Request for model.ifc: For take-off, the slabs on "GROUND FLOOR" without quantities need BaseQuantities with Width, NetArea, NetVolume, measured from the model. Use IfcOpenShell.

First a look at what the model holds.

```python
import ifcopenshell
import ifcopenshell.util.element
import ifcopenshell.util.unit

model = ifcopenshell.open("model.ifc")
print(model.schema)
for unit_type in ("LENGTHUNIT", "AREAUNIT", "VOLUMEUNIT"):
    print(unit_type, ifcopenshell.util.unit.calculate_unit_scale(model, unit_type))
storey = next(s for s in model.by_type("IfcBuildingStorey") if s.Name == "GROUND FLOOR")
slabs = [e for e in ifcopenshell.util.element.get_decomposition(storey) if e.is_a("IfcSlab")]
for e in sorted(slabs, key=lambda e: e.id()):
    print(e.id(), e.is_a(), e.Name, list(ifcopenshell.util.element.get_psets(e, qtos_only=True)), sep=" | ")
```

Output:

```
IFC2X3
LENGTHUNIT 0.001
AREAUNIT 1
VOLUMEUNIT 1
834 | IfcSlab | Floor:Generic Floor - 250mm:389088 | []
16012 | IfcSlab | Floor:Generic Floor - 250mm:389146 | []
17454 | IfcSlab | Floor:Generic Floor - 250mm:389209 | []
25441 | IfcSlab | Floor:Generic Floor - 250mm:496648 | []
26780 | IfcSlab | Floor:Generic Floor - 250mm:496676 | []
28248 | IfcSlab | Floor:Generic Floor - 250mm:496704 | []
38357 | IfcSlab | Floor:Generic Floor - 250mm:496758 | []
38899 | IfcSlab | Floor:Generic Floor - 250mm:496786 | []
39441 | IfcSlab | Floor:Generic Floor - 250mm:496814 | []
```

```python
import ifcopenshell
import ifcopenshell.api.pset
import ifcopenshell.geom
import ifcopenshell.util.element
import ifcopenshell.util.shape
import ifcopenshell.util.unit

model = ifcopenshell.open("model.ifc")
unit_scale = ifcopenshell.util.unit.calculate_unit_scale(model)
area_scale = ifcopenshell.util.unit.calculate_unit_scale(model, "AREAUNIT")
volume_scale = ifcopenshell.util.unit.calculate_unit_scale(model, "VOLUMEUNIT")
settings = ifcopenshell.geom.settings()

storey = next(s for s in model.by_type("IfcBuildingStorey") if s.Name == "GROUND FLOOR")
slabs = [e for e in ifcopenshell.util.element.get_decomposition(storey) if e.is_a("IfcSlab")]

for e in sorted(slabs, key=lambda e: e.id()):
    if ifcopenshell.util.element.get_psets(e, qtos_only=True, should_inherit=False):
        continue
    # Geometry comes back in metres, in the element's own axes.
    shape = ifcopenshell.geom.create_shape(settings, e)
    values = {
        "Width": ifcopenshell.util.shape.get_z(shape.geometry) / unit_scale,
        "NetArea": ifcopenshell.util.shape.get_footprint_area(shape.geometry) / area_scale,
        "NetVolume": ifcopenshell.util.shape.get_volume(shape.geometry) / volume_scale,
    }
    qto = ifcopenshell.api.pset.add_qto(model, product=e, name="BaseQuantities")
    ifcopenshell.api.pset.edit_qto(model, qto=qto, properties=values)
    print(e.id(), {k: round(v, 3) for k, v in values.items()})

model.write("model_edited.ifc")
```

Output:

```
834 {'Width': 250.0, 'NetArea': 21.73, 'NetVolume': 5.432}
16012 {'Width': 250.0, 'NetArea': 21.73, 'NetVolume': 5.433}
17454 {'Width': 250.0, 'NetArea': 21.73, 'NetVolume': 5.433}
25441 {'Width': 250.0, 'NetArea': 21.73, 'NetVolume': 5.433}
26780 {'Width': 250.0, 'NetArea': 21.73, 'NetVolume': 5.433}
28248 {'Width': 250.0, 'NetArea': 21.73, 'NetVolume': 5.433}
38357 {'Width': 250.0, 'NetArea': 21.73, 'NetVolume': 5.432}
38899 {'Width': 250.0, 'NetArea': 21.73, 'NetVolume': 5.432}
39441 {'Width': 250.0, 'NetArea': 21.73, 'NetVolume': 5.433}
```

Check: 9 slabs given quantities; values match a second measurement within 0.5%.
